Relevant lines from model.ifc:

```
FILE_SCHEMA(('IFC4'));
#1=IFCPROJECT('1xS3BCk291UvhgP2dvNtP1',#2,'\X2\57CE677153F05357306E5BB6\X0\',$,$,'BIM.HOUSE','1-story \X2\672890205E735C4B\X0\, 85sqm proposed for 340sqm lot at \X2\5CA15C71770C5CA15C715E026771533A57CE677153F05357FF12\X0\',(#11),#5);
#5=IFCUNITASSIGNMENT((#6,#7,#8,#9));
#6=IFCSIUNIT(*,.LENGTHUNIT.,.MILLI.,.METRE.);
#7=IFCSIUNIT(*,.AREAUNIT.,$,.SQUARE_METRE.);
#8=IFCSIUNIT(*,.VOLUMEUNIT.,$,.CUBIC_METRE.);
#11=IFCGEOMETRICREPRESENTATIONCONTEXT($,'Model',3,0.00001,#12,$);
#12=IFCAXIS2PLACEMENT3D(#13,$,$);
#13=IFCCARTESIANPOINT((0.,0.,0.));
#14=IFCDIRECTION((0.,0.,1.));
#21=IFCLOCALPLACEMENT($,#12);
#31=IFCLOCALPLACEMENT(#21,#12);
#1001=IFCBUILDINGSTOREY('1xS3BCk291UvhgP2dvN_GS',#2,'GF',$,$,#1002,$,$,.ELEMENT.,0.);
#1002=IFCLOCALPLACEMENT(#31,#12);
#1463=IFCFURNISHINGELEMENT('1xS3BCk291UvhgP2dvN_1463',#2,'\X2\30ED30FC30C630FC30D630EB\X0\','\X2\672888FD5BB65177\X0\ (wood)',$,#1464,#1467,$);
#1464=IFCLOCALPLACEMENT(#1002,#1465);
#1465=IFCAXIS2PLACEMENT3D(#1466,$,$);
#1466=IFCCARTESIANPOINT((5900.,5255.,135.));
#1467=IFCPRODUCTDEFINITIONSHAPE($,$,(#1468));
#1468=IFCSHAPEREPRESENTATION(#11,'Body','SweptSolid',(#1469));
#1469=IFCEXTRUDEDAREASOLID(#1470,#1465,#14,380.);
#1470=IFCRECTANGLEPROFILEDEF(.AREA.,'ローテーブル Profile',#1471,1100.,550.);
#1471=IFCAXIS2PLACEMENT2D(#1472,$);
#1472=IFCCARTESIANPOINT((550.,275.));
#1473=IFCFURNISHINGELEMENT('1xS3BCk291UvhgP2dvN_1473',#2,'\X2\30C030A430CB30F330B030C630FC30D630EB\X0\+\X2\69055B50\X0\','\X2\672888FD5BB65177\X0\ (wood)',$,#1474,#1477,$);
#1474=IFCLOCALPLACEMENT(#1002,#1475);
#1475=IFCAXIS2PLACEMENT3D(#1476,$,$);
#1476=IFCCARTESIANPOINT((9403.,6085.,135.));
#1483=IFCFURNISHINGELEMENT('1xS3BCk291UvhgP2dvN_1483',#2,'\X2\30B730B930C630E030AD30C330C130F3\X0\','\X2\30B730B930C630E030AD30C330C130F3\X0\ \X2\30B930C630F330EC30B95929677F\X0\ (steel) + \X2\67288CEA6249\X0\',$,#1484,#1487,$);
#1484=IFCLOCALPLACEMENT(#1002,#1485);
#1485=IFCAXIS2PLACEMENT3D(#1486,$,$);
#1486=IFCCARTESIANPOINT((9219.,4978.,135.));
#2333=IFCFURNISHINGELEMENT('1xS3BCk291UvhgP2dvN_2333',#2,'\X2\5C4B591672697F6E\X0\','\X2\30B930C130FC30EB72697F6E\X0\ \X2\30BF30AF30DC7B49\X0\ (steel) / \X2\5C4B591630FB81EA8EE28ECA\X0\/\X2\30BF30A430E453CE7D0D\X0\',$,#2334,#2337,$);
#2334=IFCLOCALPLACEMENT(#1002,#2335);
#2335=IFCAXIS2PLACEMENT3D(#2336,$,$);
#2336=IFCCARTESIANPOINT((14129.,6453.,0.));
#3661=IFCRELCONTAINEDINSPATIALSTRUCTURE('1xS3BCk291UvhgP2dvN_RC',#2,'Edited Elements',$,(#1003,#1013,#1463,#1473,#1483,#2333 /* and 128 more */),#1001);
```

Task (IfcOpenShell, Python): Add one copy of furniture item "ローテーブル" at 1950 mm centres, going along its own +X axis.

```python
import ifcopenshell
import ifcopenshell.api.geometry
import ifcopenshell.api.root
import ifcopenshell.util.element
import ifcopenshell.util.placement
import ifcopenshell.util.unit

model = ifcopenshell.open("model.ifc")
unit_scale = ifcopenshell.util.unit.calculate_unit_scale(model)


def reuse_history(source, copy):
    """copy_class also copies each property set's owner history, people and application; keep the originals."""
    for rel in copy.IsDefinedBy:
        if rel.is_a("IfcRelDefinesByProperties") and (history := rel.RelatingPropertyDefinition.OwnerHistory):
            rel.RelatingPropertyDefinition.OwnerHistory = source.OwnerHistory
            ifcopenshell.util.element.remove_deep2(model, history)


source = model.by_guid("1xS3BCk291UvhgP2dvN_1463")
base = ifcopenshell.util.placement.get_local_placement(source.ObjectPlacement)
step = base[:3, 0] * 1.95 / unit_scale

for i in range(1, 2):
    copy = ifcopenshell.api.root.copy_class(model, product=source)
    copy.Representation = ifcopenshell.util.element.copy_deep(
        model, source.Representation, exclude=["IfcGeometricRepresentationContext", "IfcRepresentationMap"]
    )
    reuse_history(source, copy)
    matrix = base.copy()
    matrix[:3, 3] += i * step
    print("added at", matrix[:3, 3].round(3) + 0.0)
    ifcopenshell.api.geometry.edit_object_placement(model, product=copy, matrix=matrix, is_si=False)

model.write("model-out.ifc")
```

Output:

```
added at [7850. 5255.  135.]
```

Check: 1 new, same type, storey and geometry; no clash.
